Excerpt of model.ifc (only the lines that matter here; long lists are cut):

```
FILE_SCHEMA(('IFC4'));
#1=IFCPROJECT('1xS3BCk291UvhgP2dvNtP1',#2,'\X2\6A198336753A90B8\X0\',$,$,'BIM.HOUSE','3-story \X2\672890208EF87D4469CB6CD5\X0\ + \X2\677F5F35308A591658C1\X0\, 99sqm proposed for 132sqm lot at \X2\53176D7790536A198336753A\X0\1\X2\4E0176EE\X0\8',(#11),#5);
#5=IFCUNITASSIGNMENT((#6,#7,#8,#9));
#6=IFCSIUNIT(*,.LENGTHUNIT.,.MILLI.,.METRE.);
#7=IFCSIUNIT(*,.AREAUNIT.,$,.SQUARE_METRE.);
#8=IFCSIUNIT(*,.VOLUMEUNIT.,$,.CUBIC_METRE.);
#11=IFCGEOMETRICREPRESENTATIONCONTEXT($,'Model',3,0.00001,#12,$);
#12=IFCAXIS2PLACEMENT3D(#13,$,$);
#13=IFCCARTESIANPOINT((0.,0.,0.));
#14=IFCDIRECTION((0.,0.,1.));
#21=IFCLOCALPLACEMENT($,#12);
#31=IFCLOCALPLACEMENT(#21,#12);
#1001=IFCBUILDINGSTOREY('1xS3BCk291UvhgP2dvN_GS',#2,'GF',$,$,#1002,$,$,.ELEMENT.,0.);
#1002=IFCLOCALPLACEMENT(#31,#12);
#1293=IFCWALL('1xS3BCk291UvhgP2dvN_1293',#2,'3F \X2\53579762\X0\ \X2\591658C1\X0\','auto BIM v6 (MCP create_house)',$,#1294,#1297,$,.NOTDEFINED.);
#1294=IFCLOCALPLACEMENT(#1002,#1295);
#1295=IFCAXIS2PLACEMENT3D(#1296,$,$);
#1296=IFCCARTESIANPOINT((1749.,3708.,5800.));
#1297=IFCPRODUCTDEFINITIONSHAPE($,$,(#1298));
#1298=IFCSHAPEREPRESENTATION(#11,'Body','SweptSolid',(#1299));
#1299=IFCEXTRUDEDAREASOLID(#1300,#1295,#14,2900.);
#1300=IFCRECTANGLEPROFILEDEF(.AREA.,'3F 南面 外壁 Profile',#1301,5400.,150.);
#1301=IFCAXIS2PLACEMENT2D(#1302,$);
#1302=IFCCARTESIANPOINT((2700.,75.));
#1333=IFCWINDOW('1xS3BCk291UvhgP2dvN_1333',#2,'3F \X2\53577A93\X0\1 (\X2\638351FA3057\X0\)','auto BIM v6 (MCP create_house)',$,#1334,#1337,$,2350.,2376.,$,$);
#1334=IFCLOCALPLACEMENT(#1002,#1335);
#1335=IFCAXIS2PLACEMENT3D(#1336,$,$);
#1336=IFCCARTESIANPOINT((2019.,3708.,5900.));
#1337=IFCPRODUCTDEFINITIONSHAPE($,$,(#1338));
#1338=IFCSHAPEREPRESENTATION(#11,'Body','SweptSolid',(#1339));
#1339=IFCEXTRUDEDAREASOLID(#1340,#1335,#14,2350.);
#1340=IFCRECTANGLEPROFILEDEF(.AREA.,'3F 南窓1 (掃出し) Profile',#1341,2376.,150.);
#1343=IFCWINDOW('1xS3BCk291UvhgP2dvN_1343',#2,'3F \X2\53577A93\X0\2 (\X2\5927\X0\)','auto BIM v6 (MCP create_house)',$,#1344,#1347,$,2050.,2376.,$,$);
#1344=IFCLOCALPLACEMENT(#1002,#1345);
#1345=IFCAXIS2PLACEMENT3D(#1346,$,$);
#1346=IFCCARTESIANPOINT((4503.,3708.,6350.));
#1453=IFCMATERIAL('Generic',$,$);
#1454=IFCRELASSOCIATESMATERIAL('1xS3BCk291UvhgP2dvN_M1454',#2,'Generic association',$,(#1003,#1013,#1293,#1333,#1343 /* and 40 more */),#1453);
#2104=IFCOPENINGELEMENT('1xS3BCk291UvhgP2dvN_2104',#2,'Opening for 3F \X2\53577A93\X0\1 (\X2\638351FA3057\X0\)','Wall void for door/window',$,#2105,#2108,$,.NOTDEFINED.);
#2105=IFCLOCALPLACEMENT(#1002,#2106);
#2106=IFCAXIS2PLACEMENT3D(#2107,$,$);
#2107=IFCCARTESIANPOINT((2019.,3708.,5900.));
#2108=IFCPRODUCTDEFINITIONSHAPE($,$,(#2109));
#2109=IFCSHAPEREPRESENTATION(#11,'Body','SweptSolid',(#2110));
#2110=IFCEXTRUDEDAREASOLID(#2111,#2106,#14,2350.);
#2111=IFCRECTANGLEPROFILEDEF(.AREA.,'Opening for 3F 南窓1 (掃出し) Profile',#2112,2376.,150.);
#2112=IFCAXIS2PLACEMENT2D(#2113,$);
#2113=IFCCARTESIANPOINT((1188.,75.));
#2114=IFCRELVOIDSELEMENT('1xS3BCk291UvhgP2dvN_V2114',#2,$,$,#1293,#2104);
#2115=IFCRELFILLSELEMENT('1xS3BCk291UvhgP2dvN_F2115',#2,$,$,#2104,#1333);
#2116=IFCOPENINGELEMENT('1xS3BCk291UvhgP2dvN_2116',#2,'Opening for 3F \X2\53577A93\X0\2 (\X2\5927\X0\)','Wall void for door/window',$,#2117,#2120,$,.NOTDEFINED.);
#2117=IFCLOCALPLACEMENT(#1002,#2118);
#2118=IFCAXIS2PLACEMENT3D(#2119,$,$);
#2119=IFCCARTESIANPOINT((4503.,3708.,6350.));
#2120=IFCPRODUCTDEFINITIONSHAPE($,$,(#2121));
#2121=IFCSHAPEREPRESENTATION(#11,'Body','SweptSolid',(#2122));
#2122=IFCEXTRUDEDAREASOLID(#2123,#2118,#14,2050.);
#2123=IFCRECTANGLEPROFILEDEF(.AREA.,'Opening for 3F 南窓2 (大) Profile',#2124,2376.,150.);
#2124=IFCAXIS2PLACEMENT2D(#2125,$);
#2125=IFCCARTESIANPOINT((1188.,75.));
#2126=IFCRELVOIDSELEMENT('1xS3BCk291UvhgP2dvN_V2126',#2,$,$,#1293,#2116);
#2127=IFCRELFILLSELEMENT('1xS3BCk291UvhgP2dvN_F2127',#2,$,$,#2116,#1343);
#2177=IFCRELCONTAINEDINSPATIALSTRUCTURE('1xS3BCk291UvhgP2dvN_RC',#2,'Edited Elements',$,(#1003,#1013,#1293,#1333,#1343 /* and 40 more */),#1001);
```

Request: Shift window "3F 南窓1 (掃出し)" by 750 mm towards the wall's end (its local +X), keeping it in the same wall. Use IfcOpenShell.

```python
import ifcopenshell
import ifcopenshell.api.geometry
import ifcopenshell.util.placement

model = ifcopenshell.open("model.ifc")

window = model.by_id(1333)
opening = window.FillsVoids[0].RelatingOpeningElement
wall = opening.VoidsElements[0].RelatingBuildingElement

wall_matrix = ifcopenshell.util.placement.get_local_placement(wall.ObjectPlacement)
shift = wall_matrix[:3, 0] * 750.0
before = ifcopenshell.util.placement.get_local_placement(window.ObjectPlacement)[:3, 3].copy()

# The window is not placed relative to its opening, so move both.
for product in (opening, window):
    matrix = ifcopenshell.util.placement.get_local_placement(product.ObjectPlacement)
    matrix[:3, 3] += shift
    ifcopenshell.api.geometry.edit_object_placement(model, product=product, matrix=matrix, is_si=False)

after = ifcopenshell.util.placement.get_local_placement(window.ObjectPlacement)[:3, 3]
print("window moved by", (after - before).round(3) + 0.0)

model.write("model-out.ifc")
```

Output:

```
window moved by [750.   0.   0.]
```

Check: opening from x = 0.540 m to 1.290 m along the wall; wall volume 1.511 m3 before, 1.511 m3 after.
